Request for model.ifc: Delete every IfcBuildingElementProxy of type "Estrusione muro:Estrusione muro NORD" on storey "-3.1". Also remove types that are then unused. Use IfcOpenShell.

First a look at what the model holds.

```python
import ifcopenshell
import ifcopenshell.util.element

model = ifcopenshell.open("model.ifc")
print(model.schema)
storey = next(s for s in model.by_type("IfcBuildingStorey") if s.Name == "-3.1")
proxies = [e for e in ifcopenshell.util.element.get_decomposition(storey) if e.is_a("IfcBuildingElementProxy")]
seen = {}
for e in proxies:
    element_type = ifcopenshell.util.element.get_type(e)
    name = element_type.Name if element_type not in (None, e) else None
    seen[name] = seen.get(name, 0) + 1
for name, count in sorted(seen.items(), key=str):
    print(count, "x", name)
```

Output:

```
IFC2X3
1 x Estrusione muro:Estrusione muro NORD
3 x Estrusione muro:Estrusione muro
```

```python
import ifcopenshell
import ifcopenshell.api.root
import ifcopenshell.util.element

model = ifcopenshell.open("model.ifc")

storey = next(s for s in model.by_type("IfcBuildingStorey") if s.Name == "-3.1")
proxies = [e for e in ifcopenshell.util.element.get_decomposition(storey) if e.is_a("IfcBuildingElementProxy")]
targets = [e for e in proxies if (t := ifcopenshell.util.element.get_type(e)) not in (None, e) and t.Name == "Estrusione muro:Estrusione muro NORD"]
types = {ifcopenshell.util.element.get_type(e) for e in targets} - {None, *targets}

for e in targets:
    ifcopenshell.api.root.remove_product(model, product=e)
print(len(targets), "removed")

unused = [t for t in types if not ifcopenshell.util.element.get_types(t)]
for t in unused:
    ifcopenshell.api.root.remove_product(model, product=t)
print(len(unused), "unused types removed")

model.write("model_updated.ifc")
```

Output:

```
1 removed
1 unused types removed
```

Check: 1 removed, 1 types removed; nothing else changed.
